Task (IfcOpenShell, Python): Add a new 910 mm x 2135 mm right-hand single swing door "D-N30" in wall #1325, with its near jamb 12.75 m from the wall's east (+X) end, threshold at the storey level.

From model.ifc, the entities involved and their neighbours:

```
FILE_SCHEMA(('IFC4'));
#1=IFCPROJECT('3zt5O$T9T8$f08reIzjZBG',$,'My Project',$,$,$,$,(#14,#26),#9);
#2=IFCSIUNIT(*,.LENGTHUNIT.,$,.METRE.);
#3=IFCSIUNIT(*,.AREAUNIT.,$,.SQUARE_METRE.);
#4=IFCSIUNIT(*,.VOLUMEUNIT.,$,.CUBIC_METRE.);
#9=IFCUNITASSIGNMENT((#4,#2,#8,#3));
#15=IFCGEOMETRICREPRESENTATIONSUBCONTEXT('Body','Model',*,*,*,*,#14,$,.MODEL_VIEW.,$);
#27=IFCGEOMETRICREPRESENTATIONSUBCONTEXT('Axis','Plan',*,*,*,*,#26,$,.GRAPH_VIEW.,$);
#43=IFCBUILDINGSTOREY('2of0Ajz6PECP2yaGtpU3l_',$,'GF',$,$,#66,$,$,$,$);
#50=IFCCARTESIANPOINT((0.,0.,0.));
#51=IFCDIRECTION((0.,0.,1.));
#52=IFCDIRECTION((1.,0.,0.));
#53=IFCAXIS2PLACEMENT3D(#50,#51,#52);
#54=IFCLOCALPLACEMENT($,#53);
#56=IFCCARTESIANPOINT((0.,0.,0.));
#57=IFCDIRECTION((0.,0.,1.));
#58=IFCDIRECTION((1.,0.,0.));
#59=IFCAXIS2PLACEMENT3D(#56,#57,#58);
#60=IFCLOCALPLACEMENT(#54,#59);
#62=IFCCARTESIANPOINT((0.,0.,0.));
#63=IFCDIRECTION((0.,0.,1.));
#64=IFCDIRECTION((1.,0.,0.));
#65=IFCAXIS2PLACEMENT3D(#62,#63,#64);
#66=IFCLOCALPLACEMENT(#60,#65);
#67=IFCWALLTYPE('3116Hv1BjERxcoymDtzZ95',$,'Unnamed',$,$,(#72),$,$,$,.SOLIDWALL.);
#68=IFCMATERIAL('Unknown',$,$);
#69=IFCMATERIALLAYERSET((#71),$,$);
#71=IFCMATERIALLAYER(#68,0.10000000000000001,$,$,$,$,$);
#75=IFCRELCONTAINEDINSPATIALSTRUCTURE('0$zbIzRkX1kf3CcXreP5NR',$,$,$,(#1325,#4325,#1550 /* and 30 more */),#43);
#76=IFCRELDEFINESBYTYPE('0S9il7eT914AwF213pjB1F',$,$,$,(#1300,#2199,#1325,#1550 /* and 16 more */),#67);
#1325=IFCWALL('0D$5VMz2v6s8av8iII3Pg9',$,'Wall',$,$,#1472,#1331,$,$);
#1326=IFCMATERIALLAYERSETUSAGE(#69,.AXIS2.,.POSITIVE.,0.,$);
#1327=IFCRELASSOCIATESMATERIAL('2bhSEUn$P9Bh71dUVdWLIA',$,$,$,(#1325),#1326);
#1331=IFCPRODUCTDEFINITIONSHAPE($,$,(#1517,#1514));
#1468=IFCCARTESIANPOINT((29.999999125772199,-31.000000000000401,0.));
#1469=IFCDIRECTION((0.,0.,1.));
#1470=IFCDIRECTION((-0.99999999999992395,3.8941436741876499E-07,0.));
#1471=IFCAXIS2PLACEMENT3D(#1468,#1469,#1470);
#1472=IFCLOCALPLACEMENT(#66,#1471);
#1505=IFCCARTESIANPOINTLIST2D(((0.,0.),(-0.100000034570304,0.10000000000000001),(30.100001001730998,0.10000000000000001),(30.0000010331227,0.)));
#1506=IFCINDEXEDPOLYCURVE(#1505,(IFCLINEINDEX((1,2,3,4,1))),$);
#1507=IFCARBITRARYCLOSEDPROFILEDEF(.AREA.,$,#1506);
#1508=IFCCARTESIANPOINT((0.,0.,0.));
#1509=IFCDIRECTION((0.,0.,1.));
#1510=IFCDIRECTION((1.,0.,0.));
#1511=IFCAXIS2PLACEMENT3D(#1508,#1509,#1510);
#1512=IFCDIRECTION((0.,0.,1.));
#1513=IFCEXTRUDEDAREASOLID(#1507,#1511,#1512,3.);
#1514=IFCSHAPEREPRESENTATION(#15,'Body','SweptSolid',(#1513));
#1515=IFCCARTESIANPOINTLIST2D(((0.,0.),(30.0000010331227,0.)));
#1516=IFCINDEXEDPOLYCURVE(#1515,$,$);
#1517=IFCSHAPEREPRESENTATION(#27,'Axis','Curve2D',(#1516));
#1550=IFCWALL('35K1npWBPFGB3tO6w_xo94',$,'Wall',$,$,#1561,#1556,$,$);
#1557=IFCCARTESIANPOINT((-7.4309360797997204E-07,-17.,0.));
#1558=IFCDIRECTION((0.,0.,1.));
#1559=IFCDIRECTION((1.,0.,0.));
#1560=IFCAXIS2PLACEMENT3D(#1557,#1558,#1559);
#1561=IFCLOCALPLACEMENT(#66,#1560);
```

```python
import numpy as np
import ifcopenshell
import ifcopenshell.api.feature
import ifcopenshell.api.geometry
import ifcopenshell.api.root
import ifcopenshell.api.spatial
import ifcopenshell.geom
import ifcopenshell.util.element
import ifcopenshell.util.placement
import ifcopenshell.util.representation
import ifcopenshell.util.shape
import ifcopenshell.util.unit

model = ifcopenshell.open("model.ifc")
unit_scale = ifcopenshell.util.unit.calculate_unit_scale(model)
settings = ifcopenshell.geom.settings()


def volume(element):
    """Net volume in cubic metres, openings subtracted."""
    shape = ifcopenshell.geom.create_shape(settings, element)
    return ifcopenshell.util.shape.get_volume(shape.geometry)


wall = model.by_id(1325)
storey = ifcopenshell.util.element.get_container(wall, ifc_class="IfcBuildingStorey")
context = ifcopenshell.util.representation.get_context(model, "Model", "Body", "MODEL_VIEW")
before = volume(wall)

width, height, from_end, sill = 0.91, 2.135, 12.75, 0.0  # metres

# The wall runs along its own X axis, and the end named is its -X end.
wall_shape = ifcopenshell.geom.create_shape(settings, wall)
x, y, z = ifcopenshell.util.shape.get_vertices(wall_shape.geometry).T
start = x.min() + from_end
face, thickness = float(y.min()), float(y.max() - y.min())
wall_matrix = ifcopenshell.util.placement.get_local_placement(wall.ObjectPlacement)
level = ifcopenshell.util.placement.get_local_placement(storey.ObjectPlacement)[2, 3]


def in_wall(x, y):
    """Placement at x, y metres in the wall's axes, at sill height."""
    matrix = wall_matrix.copy()
    matrix[:, 3] = wall_matrix @ np.array([x / unit_scale, y / unit_scale, 0.0, 1.0])
    matrix[2, 3] = level + sill / unit_scale
    return matrix


# Opening: a box that overshoots both wall faces by 50 mm.
opening = ifcopenshell.api.root.create_entity(model, ifc_class="IfcOpeningElement", predefined_type="OPENING")
box = ifcopenshell.api.geometry.add_wall_representation(
    model, context=context, length=width, height=height, thickness=thickness + 0.1
)
ifcopenshell.api.geometry.assign_representation(model, product=opening, representation=box)
ifcopenshell.api.geometry.edit_object_placement(model, product=opening, matrix=in_wall(start, face - 0.05), is_si=False)
ifcopenshell.api.feature.add_feature(model, feature=opening, element=wall)

door = ifcopenshell.api.root.create_entity(model, ifc_class="IfcDoor", name="D-N30", predefined_type="DOOR")
door.OverallWidth, door.OverallHeight = width / unit_scale, height / unit_scale
door.OperationType = "SINGLE_SWING_RIGHT"
body = ifcopenshell.api.geometry.add_door_representation(
    model,
    context=context,
    overall_width=door.OverallWidth,
    overall_height=door.OverallHeight,
    operation_type="SINGLE_SWING_RIGHT",
    lining_properties={"LiningDepth": thickness / unit_scale, "ThresholdDepth": thickness / unit_scale},
)
ifcopenshell.api.geometry.assign_representation(model, product=door, representation=body)
ifcopenshell.api.spatial.assign_container(model, products=[door], relating_structure=storey)
ifcopenshell.api.feature.add_filling(model, opening=opening, element=door)

# The lining spans the wall, so the door starts at the wall face.
ifcopenshell.api.geometry.edit_object_placement(model, product=door, matrix=in_wall(start, face), is_si=False)

after = volume(wall)

print(f"wall volume {before:.3f} -> {after:.3f} m3")

model.write("model_v2.ifc")
```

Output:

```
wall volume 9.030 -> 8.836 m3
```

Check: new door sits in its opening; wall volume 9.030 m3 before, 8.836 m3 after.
